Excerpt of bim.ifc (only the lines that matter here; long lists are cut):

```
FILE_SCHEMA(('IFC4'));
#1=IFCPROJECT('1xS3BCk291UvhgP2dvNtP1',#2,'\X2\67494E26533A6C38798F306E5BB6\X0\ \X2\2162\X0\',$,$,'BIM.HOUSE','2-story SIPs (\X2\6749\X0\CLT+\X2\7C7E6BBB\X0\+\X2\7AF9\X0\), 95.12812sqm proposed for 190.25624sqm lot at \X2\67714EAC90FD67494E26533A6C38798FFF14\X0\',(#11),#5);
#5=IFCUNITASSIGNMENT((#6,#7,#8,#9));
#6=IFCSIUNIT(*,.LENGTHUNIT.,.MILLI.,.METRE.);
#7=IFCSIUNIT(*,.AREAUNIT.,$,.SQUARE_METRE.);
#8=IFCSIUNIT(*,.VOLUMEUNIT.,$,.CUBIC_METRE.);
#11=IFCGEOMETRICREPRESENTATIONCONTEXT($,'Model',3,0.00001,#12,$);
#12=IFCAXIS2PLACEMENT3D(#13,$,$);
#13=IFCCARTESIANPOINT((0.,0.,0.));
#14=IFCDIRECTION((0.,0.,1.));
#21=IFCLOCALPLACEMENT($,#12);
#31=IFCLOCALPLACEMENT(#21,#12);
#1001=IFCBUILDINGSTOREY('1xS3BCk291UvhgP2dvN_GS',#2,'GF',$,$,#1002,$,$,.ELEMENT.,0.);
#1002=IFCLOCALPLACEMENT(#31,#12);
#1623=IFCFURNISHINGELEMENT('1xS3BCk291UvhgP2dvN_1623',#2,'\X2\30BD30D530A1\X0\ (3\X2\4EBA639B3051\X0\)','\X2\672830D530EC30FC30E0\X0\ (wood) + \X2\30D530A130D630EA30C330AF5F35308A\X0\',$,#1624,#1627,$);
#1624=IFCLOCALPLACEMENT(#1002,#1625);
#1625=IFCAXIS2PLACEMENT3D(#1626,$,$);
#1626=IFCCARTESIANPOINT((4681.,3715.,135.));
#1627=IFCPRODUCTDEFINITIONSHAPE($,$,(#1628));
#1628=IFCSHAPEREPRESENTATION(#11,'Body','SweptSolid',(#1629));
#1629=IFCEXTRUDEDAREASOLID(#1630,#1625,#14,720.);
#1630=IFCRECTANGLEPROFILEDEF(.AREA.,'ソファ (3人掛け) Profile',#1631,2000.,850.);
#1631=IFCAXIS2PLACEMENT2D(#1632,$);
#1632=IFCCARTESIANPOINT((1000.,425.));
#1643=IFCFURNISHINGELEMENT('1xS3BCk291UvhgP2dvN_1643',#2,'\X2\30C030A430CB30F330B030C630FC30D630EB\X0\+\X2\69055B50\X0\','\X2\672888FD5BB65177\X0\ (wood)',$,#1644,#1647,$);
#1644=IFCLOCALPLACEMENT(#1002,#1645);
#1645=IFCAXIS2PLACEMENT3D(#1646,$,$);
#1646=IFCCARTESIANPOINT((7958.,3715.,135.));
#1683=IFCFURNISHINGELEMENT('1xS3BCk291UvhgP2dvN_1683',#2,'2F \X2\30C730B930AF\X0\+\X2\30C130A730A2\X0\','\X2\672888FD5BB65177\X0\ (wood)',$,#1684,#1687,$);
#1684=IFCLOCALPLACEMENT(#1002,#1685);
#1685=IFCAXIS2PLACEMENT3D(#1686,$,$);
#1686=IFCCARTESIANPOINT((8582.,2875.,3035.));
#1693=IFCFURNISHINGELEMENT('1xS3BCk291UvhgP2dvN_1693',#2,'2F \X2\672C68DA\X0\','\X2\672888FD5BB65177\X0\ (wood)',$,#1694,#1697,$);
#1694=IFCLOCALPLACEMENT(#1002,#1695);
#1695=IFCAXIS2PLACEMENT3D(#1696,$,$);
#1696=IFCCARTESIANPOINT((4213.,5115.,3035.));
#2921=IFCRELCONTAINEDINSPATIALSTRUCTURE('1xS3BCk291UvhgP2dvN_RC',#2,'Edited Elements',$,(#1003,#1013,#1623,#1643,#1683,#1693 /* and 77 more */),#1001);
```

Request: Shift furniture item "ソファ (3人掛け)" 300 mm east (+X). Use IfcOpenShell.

```python
import ifcopenshell
import ifcopenshell.api.geometry
import ifcopenshell.util.placement
import ifcopenshell.util.unit

model = ifcopenshell.open("bim.ifc")
unit_scale = ifcopenshell.util.unit.calculate_unit_scale(model)

item = model.by_id(1623)
matrix = ifcopenshell.util.placement.get_local_placement(item.ObjectPlacement)
matrix[0, 3] += 0.3 / unit_scale
ifcopenshell.api.geometry.edit_object_placement(model, product=item, matrix=matrix, is_si=False)

print(ifcopenshell.util.placement.get_local_placement(item.ObjectPlacement).round(3) + 0.0)

model.write("bim_rev.ifc")
```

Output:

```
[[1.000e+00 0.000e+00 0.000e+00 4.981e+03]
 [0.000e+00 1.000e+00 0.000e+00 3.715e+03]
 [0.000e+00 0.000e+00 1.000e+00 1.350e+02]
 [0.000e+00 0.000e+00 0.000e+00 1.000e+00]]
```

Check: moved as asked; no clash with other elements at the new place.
